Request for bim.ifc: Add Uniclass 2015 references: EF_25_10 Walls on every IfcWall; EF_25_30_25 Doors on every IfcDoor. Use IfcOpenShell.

First a look at what the model holds.

```python
import ifcopenshell

model = ifcopenshell.open("bim.ifc")
print(model.schema)
print("classifications:", [c.Name for c in model.by_type("IfcClassification")])
for ifc_class in ("IfcDoor", "IfcRoof", "IfcStair", "IfcWall", "IfcWindow"):
    print(ifc_class, len(model.by_type(ifc_class)))
```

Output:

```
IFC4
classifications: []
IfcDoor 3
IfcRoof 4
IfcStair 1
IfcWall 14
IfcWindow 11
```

```python
import ifcopenshell
import ifcopenshell.api.classification

model = ifcopenshell.open("bim.ifc")

system = ifcopenshell.api.classification.add_classification(model, classification="Uniclass 2015")

codes = {
    "IfcWall": ("EF_25_10", "Walls"),
    "IfcDoor": ("EF_25_30_25", "Doors"),
}
for ifc_class, (code, name) in codes.items():
    products = model.by_type(ifc_class)
    ifcopenshell.api.classification.add_reference(
        model, products=products, classification=system, identification=code, name=name
    )
    print(code, len(products))

model.write("bim_rev.ifc")
```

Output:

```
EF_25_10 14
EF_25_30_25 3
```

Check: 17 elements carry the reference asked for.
